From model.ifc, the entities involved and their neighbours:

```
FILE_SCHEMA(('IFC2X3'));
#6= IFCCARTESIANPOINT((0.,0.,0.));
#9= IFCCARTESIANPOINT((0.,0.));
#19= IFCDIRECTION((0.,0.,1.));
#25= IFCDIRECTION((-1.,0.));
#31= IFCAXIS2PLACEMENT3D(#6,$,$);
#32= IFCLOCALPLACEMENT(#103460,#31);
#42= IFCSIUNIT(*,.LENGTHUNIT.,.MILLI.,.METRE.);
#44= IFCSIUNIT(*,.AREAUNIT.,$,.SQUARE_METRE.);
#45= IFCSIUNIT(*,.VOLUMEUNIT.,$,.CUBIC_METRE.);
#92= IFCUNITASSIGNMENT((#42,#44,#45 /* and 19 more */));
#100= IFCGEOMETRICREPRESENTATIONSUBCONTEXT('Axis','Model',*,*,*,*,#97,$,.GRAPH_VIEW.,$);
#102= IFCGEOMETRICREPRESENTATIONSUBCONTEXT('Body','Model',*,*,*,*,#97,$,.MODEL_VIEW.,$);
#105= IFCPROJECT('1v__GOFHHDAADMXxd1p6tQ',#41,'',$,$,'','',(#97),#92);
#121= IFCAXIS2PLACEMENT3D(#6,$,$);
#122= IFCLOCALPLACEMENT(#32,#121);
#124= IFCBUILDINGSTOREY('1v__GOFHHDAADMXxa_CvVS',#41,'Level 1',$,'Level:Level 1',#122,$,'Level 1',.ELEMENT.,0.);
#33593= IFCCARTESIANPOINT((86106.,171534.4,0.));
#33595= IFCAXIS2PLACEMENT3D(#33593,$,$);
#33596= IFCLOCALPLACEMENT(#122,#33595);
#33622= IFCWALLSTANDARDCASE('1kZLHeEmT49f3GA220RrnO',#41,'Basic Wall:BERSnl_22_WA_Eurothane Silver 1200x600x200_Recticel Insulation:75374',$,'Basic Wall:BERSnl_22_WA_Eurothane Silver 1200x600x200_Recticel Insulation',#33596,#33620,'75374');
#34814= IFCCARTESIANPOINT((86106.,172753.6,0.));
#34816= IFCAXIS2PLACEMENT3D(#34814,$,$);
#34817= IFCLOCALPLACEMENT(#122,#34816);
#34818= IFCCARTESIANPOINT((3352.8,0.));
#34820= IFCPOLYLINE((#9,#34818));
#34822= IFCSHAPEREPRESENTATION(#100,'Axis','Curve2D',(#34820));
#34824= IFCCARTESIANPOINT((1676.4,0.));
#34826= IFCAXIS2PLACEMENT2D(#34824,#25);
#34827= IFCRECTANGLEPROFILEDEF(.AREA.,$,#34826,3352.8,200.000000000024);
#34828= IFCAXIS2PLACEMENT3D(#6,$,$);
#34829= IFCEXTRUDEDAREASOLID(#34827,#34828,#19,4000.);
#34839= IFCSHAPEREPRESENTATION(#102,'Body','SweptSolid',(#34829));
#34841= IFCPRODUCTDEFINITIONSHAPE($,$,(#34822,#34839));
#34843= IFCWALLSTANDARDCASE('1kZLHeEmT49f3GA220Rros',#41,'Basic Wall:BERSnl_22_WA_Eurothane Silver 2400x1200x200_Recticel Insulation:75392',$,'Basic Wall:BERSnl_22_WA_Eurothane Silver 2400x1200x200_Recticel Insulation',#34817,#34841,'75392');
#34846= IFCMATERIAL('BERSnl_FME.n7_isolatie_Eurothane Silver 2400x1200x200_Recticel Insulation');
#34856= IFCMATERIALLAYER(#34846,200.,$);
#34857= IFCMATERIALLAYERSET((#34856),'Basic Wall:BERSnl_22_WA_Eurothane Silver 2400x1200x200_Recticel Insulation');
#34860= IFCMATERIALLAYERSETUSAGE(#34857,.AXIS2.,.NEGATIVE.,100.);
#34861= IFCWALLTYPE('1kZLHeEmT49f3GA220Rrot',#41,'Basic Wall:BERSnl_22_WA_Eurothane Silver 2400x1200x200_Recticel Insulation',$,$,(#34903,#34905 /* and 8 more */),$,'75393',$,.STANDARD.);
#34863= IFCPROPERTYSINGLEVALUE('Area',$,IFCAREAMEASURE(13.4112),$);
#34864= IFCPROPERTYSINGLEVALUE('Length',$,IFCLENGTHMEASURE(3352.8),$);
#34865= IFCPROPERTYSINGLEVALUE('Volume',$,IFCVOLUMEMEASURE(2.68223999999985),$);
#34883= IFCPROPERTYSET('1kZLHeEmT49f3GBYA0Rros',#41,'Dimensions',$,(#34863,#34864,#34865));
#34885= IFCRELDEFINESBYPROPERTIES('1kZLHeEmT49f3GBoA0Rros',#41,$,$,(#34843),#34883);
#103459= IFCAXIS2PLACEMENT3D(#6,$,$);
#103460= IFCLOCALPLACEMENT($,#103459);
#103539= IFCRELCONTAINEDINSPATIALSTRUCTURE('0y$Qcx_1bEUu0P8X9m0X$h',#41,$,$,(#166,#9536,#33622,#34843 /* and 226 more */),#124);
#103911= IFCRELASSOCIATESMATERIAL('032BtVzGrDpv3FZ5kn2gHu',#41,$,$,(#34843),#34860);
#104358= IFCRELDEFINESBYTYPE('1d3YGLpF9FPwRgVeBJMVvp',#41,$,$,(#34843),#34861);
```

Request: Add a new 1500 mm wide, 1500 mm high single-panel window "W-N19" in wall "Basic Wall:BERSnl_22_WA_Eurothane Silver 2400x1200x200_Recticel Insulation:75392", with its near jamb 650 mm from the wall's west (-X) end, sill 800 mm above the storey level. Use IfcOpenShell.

```python
import numpy as np
import ifcopenshell
import ifcopenshell.api.feature
import ifcopenshell.api.geometry
import ifcopenshell.api.pset
import ifcopenshell.api.root
import ifcopenshell.api.spatial
import ifcopenshell.api.type
import ifcopenshell.geom
import ifcopenshell.util.element
import ifcopenshell.util.placement
import ifcopenshell.util.representation
import ifcopenshell.util.shape
import ifcopenshell.util.unit

model = ifcopenshell.open("model.ifc")
unit_scale = ifcopenshell.util.unit.calculate_unit_scale(model)
area_scale = ifcopenshell.util.unit.calculate_unit_scale(model, "AREAUNIT")
volume_scale = ifcopenshell.util.unit.calculate_unit_scale(model, "VOLUMEUNIT")
settings = ifcopenshell.geom.settings()


def volume(element):
    """Net volume in cubic metres, openings subtracted."""
    shape = ifcopenshell.geom.create_shape(settings, element)
    return ifcopenshell.util.shape.get_volume(shape.geometry)


wall = model.by_id(34843)
storey = ifcopenshell.util.element.get_container(wall, ifc_class="IfcBuildingStorey")
context = ifcopenshell.util.representation.get_context(model, "Model", "Body", "MODEL_VIEW")
before = volume(wall)

width, height, from_end, sill = 1.5, 1.5, 0.65, 0.8  # metres

# The wall runs along its own X axis, and the end named is its -X end.
wall_shape = ifcopenshell.geom.create_shape(settings, wall)
x, y, z = ifcopenshell.util.shape.get_vertices(wall_shape.geometry).T
start = x.min() + from_end
face, thickness = float(y.min()), float(y.max() - y.min())
wall_matrix = ifcopenshell.util.placement.get_local_placement(wall.ObjectPlacement)
level = ifcopenshell.util.placement.get_local_placement(storey.ObjectPlacement)[2, 3]


def in_wall(x, y):
    """Placement at x, y metres in the wall's axes, at sill height."""
    matrix = wall_matrix.copy()
    matrix[:, 3] = wall_matrix @ np.array([x / unit_scale, y / unit_scale, 0.0, 1.0])
    matrix[2, 3] = level + sill / unit_scale
    return matrix


# Opening: a box that overshoots both wall faces by 50 mm.
opening = ifcopenshell.api.root.create_entity(model, ifc_class="IfcOpeningElement")
box = ifcopenshell.api.geometry.add_wall_representation(
    model, context=context, length=width, height=height, thickness=thickness + 0.1
)
ifcopenshell.api.geometry.assign_representation(model, product=opening, representation=box)
ifcopenshell.api.geometry.edit_object_placement(model, product=opening, matrix=in_wall(start, face - 0.05), is_si=False)
ifcopenshell.api.feature.add_feature(model, feature=opening, element=wall)

window = ifcopenshell.api.root.create_entity(model, ifc_class="IfcWindow", name="W-N19")
window.OverallWidth, window.OverallHeight = width / unit_scale, height / unit_scale
body = ifcopenshell.api.geometry.add_window_representation(
    model,
    context=context,
    overall_width=window.OverallWidth,
    overall_height=window.OverallHeight,
    partition_type="SINGLE_PANEL",
)
ifcopenshell.api.geometry.assign_representation(model, product=window, representation=body)
ifcopenshell.api.spatial.assign_container(model, products=[window], relating_structure=storey)
fills = ifcopenshell.api.feature.add_filling(model, opening=opening, element=window)
fills.OwnerHistory = window.OwnerHistory  # required in IFC2X3

# IFC2X3 keeps the operation on the window style.
style = ifcopenshell.api.root.create_entity(model, ifc_class="IfcWindowStyle", name="W-N19")
style.OperationType, style.ConstructionType = "SINGLE_PANEL", "NOTDEFINED"
style.ParameterTakesPrecedence = style.Sizeable = False
ifcopenshell.api.type.assign_type(model, related_objects=[window], relating_type=style)

# Centre the window in the wall's thickness.
ifcopenshell.api.geometry.edit_object_placement(model, product=window, matrix=in_wall(start, face), is_si=False)
window_shape = ifcopenshell.geom.create_shape(settings, window)
depth = ifcopenshell.util.shape.get_vertices(window_shape.geometry)[:, 1]
offset = face + thickness / 2 - (depth.min() + depth.max()) / 2
ifcopenshell.api.geometry.edit_object_placement(model, product=window, matrix=in_wall(start, offset), is_si=False)

after = volume(wall)

# Update the wall's stored quantities.
pset = model.by_id(ifcopenshell.util.element.get_pset(wall, "Dimensions", should_inherit=False)["id"])
ifcopenshell.api.pset.edit_pset(model, pset=pset, properties={
    "Area": model.create_entity("IfcAreaMeasure", after / thickness / area_scale),
    "Volume": model.create_entity("IfcVolumeMeasure", after / volume_scale),
})

print(f"wall volume {before:.3f} -> {after:.3f} m3")

model.write("model_v2.ifc")
```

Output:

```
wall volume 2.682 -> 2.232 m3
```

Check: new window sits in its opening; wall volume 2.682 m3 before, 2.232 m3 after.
